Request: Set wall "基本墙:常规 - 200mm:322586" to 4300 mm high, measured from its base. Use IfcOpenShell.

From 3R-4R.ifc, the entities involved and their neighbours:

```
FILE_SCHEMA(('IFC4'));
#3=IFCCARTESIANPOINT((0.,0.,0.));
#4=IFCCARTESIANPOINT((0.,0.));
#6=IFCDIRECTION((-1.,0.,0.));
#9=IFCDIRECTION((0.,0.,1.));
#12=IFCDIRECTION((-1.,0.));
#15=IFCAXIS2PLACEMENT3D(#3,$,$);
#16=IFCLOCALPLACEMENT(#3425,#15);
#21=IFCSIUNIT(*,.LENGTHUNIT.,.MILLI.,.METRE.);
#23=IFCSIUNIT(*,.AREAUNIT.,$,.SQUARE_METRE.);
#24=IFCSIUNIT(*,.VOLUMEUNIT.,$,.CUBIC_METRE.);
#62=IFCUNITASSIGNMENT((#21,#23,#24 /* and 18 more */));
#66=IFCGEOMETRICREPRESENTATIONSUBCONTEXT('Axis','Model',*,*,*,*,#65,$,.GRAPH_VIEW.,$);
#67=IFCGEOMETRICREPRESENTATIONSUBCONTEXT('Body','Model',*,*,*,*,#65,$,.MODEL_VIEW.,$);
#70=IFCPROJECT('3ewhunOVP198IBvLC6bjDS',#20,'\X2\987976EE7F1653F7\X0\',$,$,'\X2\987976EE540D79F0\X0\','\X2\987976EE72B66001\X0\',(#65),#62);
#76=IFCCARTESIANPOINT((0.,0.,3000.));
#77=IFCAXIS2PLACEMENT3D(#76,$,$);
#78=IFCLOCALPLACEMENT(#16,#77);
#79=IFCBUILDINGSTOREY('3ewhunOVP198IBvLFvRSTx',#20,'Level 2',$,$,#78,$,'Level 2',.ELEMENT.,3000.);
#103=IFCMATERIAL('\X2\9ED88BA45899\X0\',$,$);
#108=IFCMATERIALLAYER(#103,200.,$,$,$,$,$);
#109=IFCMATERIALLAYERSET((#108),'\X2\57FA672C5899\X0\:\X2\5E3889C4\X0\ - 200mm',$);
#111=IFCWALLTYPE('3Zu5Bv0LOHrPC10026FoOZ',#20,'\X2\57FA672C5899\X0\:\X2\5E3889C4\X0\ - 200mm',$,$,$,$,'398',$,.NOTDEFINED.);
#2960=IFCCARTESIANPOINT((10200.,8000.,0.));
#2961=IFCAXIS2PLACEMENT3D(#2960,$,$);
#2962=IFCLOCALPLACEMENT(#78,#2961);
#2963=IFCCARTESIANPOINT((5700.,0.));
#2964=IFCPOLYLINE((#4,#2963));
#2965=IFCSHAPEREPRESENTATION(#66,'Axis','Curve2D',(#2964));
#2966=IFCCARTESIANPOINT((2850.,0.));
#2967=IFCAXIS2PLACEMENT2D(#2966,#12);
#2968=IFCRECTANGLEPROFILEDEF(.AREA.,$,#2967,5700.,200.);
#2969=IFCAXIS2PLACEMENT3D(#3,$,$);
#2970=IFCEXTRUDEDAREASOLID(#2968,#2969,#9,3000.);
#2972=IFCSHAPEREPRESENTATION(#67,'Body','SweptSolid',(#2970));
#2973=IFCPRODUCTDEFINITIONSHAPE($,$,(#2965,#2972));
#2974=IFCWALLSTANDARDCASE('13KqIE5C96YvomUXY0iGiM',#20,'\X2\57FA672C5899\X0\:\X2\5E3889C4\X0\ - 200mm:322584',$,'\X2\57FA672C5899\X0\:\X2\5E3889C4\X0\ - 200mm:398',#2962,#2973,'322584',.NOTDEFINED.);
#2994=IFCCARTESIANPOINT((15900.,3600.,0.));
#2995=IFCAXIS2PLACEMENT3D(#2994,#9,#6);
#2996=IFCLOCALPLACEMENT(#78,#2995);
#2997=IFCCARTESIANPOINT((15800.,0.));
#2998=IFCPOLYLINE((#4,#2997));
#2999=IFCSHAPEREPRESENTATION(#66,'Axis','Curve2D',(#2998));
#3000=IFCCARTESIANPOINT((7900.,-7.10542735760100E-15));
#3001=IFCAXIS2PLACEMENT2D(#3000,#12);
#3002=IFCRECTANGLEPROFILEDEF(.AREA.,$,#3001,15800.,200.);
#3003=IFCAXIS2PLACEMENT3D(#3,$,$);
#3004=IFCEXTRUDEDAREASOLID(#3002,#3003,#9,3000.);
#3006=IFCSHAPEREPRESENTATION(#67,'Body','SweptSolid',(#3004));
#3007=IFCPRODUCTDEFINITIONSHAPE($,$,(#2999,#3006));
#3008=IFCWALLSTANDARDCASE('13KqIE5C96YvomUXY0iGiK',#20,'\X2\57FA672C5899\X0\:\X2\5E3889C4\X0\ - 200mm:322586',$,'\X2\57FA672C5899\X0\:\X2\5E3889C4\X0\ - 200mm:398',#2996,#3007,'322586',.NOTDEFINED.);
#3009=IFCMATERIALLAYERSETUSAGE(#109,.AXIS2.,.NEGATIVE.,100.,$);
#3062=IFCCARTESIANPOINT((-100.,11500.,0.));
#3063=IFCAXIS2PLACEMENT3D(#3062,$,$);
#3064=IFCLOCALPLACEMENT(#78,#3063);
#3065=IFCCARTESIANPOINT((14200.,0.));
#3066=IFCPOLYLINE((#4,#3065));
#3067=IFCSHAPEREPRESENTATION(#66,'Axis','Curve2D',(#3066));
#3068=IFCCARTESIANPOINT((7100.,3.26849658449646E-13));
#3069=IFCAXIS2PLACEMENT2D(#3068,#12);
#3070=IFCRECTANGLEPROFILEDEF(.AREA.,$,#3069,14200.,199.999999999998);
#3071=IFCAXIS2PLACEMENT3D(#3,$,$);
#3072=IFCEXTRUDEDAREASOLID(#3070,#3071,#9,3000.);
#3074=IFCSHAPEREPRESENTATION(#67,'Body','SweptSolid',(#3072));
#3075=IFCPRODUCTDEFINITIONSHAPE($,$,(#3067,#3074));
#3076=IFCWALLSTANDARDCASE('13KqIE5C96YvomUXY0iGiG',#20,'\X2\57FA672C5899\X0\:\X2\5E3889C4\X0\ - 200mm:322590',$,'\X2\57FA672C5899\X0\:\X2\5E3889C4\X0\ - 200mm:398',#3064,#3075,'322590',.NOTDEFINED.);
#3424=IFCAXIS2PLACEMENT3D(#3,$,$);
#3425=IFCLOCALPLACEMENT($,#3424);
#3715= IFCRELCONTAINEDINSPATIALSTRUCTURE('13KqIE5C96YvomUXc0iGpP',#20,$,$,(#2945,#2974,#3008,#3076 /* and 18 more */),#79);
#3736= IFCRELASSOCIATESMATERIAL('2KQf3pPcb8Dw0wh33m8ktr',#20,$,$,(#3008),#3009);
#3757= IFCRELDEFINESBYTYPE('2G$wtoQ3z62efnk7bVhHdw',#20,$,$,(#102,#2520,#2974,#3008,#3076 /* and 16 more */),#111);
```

```python
import ifcopenshell
import ifcopenshell.geom
import ifcopenshell.util.representation
import ifcopenshell.util.shape
import ifcopenshell.util.unit

model = ifcopenshell.open("3R-4R.ifc")
unit_scale = ifcopenshell.util.unit.calculate_unit_scale(model)
settings = ifcopenshell.geom.settings()


def volume(element):
    """Net volume in cubic metres, openings subtracted."""
    shape = ifcopenshell.geom.create_shape(settings, element)
    return ifcopenshell.util.shape.get_volume(shape.geometry)


wall = model.by_guid("13KqIE5C96YvomUXY0iGiK")
before = volume(wall)

body = ifcopenshell.util.representation.get_representation(wall, "Model", "Body")
solid = body.Items[0]
old_height = solid.Depth
solid.Depth = 4.3 / unit_scale
after = volume(wall)

print(f"height {old_height:g} -> {solid.Depth:g}, volume {before:.3f} -> {after:.3f} m3")

model.write("3R-4R_v2.ifc")
```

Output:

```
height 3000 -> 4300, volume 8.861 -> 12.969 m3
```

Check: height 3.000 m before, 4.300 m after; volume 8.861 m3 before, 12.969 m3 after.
